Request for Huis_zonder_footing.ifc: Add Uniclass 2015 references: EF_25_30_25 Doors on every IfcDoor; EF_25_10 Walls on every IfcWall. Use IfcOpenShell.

First a look at what the model holds.

```python
import ifcopenshell

model = ifcopenshell.open("Huis_zonder_footing.ifc")
print(model.schema)
print("classifications:", [c.Name for c in model.by_type("IfcClassification")])
for ifc_class in ("IfcDoor", "IfcRoof", "IfcStair", "IfcWall", "IfcWindow"):
    print(ifc_class, len(model.by_type(ifc_class)))
```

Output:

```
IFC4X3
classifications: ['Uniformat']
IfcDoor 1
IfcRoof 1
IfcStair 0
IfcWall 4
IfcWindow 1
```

```python
import ifcopenshell
import ifcopenshell.api.classification

model = ifcopenshell.open("Huis_zonder_footing.ifc")

system = ifcopenshell.api.classification.add_classification(model, classification="Uniclass 2015")

codes = {
    "IfcDoor": ("EF_25_30_25", "Doors"),
    "IfcWall": ("EF_25_10", "Walls"),
}
for ifc_class, (code, name) in codes.items():
    products = model.by_type(ifc_class)
    ifcopenshell.api.classification.add_reference(
        model, products=products, classification=system, identification=code, name=name
    )
    print(code, len(products))

model.write("Huis_zonder_footing_edited.ifc")
```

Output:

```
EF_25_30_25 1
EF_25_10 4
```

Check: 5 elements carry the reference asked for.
